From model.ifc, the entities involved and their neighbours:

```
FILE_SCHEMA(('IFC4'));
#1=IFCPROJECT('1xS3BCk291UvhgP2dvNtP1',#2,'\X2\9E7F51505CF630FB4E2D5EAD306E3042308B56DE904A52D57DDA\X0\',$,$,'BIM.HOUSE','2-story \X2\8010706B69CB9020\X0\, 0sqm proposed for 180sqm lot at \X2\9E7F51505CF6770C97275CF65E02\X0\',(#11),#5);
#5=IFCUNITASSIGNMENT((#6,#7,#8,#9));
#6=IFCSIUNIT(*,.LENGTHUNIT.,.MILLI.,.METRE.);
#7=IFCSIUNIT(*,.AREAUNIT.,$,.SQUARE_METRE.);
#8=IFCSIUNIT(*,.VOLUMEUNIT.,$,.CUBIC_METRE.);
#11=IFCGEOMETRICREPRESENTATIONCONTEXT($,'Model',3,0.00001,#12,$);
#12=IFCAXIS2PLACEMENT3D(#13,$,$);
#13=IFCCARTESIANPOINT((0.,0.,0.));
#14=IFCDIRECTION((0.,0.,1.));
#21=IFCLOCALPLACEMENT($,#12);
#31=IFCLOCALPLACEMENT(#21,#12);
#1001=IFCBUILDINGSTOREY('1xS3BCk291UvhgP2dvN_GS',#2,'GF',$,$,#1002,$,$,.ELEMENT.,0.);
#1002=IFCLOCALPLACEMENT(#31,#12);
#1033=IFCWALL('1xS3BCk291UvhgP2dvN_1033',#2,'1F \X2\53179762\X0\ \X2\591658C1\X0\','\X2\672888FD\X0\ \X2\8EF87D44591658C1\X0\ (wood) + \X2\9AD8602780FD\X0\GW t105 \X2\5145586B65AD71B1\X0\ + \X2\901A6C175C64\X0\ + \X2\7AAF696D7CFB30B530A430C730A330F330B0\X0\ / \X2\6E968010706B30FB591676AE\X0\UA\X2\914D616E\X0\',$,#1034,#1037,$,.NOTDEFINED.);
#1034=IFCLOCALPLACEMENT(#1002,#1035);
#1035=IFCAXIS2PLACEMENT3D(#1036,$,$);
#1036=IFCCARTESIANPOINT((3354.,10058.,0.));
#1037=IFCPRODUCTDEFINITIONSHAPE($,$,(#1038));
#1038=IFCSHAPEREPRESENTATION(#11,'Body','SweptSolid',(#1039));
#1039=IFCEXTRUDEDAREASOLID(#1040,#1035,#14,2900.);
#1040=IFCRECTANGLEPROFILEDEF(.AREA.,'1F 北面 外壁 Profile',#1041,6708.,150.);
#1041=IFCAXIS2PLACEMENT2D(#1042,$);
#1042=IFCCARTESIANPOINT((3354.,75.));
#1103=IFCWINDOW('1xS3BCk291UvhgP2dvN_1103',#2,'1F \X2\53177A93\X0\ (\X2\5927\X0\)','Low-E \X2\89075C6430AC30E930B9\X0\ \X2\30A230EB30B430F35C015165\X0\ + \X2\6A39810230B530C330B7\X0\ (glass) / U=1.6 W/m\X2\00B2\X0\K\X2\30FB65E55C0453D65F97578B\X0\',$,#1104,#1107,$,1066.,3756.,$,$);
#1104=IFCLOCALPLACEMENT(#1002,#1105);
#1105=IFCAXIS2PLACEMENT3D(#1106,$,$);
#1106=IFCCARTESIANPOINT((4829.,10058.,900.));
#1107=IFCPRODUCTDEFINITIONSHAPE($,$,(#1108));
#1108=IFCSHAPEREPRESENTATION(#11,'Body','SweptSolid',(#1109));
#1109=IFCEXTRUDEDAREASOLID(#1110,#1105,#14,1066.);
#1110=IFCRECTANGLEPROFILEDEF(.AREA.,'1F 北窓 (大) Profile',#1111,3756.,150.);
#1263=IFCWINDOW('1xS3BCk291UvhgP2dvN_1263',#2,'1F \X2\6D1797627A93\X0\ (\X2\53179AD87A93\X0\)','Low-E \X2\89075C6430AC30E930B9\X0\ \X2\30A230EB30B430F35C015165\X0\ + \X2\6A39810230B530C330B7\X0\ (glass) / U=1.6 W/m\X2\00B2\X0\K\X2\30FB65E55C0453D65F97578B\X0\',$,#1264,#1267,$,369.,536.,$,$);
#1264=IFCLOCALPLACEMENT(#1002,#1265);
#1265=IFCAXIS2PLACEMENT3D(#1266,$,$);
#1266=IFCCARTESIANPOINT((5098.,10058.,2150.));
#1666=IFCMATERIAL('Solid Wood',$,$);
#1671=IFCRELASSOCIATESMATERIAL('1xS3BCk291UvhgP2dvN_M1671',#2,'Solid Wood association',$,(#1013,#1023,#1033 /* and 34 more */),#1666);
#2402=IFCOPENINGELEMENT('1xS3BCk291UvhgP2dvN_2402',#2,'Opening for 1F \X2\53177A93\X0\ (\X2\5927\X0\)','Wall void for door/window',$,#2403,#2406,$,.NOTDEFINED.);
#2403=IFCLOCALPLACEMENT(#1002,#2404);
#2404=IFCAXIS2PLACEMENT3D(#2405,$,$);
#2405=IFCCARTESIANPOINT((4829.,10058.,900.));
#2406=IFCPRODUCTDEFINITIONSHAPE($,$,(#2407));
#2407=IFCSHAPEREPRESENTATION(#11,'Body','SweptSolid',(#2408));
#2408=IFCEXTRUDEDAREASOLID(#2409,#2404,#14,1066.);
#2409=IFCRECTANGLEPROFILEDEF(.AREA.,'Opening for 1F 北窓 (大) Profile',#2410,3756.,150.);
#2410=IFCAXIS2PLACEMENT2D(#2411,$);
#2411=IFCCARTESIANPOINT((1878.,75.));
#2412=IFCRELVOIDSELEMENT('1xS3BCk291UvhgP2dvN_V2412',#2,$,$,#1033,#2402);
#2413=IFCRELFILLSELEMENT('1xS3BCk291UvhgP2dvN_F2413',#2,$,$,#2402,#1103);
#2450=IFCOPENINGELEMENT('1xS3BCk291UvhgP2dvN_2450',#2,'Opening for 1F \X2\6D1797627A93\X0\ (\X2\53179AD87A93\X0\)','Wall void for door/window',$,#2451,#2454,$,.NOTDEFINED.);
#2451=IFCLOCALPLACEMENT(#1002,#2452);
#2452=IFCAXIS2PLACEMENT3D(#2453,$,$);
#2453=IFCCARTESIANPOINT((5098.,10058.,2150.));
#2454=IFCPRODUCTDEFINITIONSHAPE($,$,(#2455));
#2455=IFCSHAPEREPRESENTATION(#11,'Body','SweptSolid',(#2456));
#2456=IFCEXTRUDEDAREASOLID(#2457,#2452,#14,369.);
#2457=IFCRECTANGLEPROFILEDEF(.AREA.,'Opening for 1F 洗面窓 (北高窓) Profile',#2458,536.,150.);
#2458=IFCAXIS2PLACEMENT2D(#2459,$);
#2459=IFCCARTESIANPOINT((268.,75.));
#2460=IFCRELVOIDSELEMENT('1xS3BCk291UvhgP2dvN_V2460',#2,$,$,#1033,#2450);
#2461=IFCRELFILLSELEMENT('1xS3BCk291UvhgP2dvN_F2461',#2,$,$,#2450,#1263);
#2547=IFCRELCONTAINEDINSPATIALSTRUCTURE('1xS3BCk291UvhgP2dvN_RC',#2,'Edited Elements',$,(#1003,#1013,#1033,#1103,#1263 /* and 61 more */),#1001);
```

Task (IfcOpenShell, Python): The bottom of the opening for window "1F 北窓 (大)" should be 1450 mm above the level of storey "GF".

```python
import numpy as np
import ifcopenshell
import ifcopenshell.api.geometry
import ifcopenshell.geom
import ifcopenshell.util.element
import ifcopenshell.util.placement
import ifcopenshell.util.shape
import ifcopenshell.util.unit

model = ifcopenshell.open("model.ifc")
unit_scale = ifcopenshell.util.unit.calculate_unit_scale(model)

window = model.by_guid("1xS3BCk291UvhgP2dvN_1103")
opening = window.FillsVoids[0].RelatingOpeningElement
storey = ifcopenshell.util.element.get_container(window, ifc_class="IfcBuildingStorey")
level = ifcopenshell.util.placement.get_local_placement(storey.ObjectPlacement)[2, 3]

# The opening's origin need not be at the sill, so measure its lowest point.
shape = ifcopenshell.geom.create_shape(ifcopenshell.geom.settings(), opening)
bottom = ifcopenshell.util.shape.get_shape_bottom_elevation(shape, shape.geometry) / unit_scale
dz = level + 1.45 / unit_scale - bottom

shift = np.array([0.0, 0.0, dz])
# The window is not placed relative to its opening, so move both.
for product in (opening, window):
    matrix = ifcopenshell.util.placement.get_local_placement(product.ObjectPlacement)
    matrix[:3, 3] += shift
    ifcopenshell.api.geometry.edit_object_placement(model, product=product, matrix=matrix, is_si=False)

print(f"moved by {dz * unit_scale:+.3f} m")

model.write("model-out.ifc")
```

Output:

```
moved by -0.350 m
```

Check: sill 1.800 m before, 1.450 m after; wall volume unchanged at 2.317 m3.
